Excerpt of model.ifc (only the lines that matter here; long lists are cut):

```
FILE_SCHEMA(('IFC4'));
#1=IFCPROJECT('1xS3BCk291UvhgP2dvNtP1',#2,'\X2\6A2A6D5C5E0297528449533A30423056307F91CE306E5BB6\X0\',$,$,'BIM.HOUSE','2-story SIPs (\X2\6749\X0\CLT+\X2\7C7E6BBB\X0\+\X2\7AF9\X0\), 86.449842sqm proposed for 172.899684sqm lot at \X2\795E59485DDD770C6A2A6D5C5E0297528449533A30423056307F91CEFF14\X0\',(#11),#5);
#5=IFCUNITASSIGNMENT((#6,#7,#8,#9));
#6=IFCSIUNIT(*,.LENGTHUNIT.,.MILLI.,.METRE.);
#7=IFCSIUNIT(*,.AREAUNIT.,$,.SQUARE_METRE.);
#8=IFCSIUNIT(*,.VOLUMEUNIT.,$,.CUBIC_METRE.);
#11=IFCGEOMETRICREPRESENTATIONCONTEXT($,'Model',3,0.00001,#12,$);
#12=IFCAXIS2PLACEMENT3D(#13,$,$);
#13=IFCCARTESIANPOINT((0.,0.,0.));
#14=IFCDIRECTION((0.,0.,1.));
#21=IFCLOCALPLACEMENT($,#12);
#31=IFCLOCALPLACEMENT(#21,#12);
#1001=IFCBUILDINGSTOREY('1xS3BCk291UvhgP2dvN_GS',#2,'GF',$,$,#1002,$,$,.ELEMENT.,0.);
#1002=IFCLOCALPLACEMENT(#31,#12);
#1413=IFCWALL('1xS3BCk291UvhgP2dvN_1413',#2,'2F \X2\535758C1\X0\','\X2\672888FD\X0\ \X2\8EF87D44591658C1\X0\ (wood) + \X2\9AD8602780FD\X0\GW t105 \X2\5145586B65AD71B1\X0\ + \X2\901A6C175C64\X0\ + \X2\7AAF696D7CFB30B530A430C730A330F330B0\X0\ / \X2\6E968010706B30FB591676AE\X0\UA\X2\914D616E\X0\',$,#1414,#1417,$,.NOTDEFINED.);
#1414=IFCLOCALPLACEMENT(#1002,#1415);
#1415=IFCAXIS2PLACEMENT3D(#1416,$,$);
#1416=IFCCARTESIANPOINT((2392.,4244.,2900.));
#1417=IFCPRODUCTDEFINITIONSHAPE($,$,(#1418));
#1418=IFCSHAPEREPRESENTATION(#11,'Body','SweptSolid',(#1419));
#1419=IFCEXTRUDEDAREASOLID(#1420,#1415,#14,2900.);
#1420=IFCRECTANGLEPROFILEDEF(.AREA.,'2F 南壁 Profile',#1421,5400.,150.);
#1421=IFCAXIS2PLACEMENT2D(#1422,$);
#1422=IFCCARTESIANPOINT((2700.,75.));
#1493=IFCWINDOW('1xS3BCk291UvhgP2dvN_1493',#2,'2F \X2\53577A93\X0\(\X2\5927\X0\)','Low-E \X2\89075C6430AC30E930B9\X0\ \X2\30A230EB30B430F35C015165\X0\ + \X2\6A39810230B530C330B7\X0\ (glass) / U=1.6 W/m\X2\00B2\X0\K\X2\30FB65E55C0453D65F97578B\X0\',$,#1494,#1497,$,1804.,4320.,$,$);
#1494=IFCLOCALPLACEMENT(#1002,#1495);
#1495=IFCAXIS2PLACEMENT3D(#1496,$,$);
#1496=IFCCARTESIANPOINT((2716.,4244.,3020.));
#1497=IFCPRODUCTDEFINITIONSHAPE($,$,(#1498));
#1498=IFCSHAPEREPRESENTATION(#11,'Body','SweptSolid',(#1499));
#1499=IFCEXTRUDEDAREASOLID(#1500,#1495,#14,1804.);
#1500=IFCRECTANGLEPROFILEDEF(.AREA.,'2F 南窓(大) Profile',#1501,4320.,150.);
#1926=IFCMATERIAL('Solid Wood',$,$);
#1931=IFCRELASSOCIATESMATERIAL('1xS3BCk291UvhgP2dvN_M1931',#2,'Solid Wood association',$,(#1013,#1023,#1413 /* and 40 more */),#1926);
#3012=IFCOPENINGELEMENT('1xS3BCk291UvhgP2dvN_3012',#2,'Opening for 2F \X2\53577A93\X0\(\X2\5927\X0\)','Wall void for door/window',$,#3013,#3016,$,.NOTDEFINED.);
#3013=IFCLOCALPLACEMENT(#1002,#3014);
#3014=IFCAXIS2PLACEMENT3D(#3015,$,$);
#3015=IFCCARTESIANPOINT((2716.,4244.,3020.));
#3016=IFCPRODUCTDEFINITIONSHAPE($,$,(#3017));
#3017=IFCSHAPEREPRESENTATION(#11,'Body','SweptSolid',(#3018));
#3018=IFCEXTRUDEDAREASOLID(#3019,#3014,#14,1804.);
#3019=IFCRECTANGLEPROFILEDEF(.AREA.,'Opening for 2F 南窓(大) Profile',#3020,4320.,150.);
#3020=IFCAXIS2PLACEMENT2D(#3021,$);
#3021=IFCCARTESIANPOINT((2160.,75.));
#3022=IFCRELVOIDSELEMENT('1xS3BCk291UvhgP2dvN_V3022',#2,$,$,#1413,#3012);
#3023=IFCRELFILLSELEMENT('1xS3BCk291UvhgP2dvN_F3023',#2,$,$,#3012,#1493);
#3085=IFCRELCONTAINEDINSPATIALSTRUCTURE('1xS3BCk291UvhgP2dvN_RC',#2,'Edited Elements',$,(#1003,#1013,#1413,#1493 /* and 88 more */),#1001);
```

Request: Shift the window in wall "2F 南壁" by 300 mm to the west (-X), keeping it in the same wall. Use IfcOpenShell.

```python
import ifcopenshell
import ifcopenshell.api.geometry
import ifcopenshell.util.placement
import ifcopenshell.util.unit

model = ifcopenshell.open("model.ifc")
unit_scale = ifcopenshell.util.unit.calculate_unit_scale(model)

window = model.by_id(1493)
opening = window.FillsVoids[0].RelatingOpeningElement
wall = opening.VoidsElements[0].RelatingBuildingElement

wall_matrix = ifcopenshell.util.placement.get_local_placement(wall.ObjectPlacement)
shift = wall_matrix[:3, 0] * -0.3 / unit_scale
before = ifcopenshell.util.placement.get_local_placement(window.ObjectPlacement)[:3, 3].copy()

# The window is not placed relative to its opening, so move both.
for product in (opening, window):
    matrix = ifcopenshell.util.placement.get_local_placement(product.ObjectPlacement)
    matrix[:3, 3] += shift
    ifcopenshell.api.geometry.edit_object_placement(model, product=product, matrix=matrix, is_si=False)

after = ifcopenshell.util.placement.get_local_placement(window.ObjectPlacement)[:3, 3]
print("window moved by", (after - before).round(3) + 0.0)

model.write("model_updated.ifc")
```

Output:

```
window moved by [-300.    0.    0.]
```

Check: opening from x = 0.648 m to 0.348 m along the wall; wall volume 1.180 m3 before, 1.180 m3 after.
